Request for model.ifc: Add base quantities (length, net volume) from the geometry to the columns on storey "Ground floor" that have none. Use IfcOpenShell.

First a look at what the model holds.

```python
import ifcopenshell
import ifcopenshell.util.element
import ifcopenshell.util.unit

model = ifcopenshell.open("model.ifc")
print(model.schema)
for unit_type in ("LENGTHUNIT", "AREAUNIT", "VOLUMEUNIT"):
    print(unit_type, ifcopenshell.util.unit.calculate_unit_scale(model, unit_type))
storey = next(s for s in model.by_type("IfcBuildingStorey") if s.Name == "Ground floor")
columns = [e for e in ifcopenshell.util.element.get_decomposition(storey) if e.is_a("IfcColumn")]
for e in sorted(columns, key=lambda e: e.id()):
    print(e.id(), e.is_a(), e.Name, list(ifcopenshell.util.element.get_psets(e, qtos_only=True)), sep=" | ")
```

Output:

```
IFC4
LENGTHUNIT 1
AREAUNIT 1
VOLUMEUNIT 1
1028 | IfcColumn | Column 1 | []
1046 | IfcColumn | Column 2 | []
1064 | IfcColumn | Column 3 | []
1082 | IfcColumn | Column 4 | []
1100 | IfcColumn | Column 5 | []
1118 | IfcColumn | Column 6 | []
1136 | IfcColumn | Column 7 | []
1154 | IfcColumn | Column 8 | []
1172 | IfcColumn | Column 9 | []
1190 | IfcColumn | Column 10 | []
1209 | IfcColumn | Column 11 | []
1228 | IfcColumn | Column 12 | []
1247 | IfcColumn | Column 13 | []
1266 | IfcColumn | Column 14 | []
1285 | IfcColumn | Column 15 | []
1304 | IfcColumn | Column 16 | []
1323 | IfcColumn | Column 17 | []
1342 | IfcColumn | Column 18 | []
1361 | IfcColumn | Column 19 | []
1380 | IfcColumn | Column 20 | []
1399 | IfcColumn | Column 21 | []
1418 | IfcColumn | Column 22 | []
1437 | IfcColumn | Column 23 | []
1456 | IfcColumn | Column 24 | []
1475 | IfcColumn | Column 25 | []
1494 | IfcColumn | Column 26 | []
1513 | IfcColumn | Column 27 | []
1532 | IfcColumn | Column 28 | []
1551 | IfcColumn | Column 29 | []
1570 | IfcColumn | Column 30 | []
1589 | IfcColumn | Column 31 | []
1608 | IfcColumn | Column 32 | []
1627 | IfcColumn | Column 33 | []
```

```python
import ifcopenshell
import ifcopenshell.api.pset
import ifcopenshell.geom
import ifcopenshell.util.element
import ifcopenshell.util.shape
import ifcopenshell.util.unit

model = ifcopenshell.open("model.ifc")
unit_scale = ifcopenshell.util.unit.calculate_unit_scale(model)
volume_scale = ifcopenshell.util.unit.calculate_unit_scale(model, "VOLUMEUNIT")
settings = ifcopenshell.geom.settings()

storey = next(s for s in model.by_type("IfcBuildingStorey") if s.Name == "Ground floor")
columns = [e for e in ifcopenshell.util.element.get_decomposition(storey) if e.is_a("IfcColumn")]

for e in sorted(columns, key=lambda e: e.id()):
    if ifcopenshell.util.element.get_psets(e, qtos_only=True, should_inherit=False):
        continue
    # Geometry comes back in metres, in the element's own axes.
    shape = ifcopenshell.geom.create_shape(settings, e)
    values = {
        "Length": ifcopenshell.util.shape.get_z(shape.geometry) / unit_scale,
        "NetVolume": ifcopenshell.util.shape.get_volume(shape.geometry) / volume_scale,
    }
    qto = ifcopenshell.api.pset.add_qto(model, product=e, name="Qto_ColumnBaseQuantities")
    ifcopenshell.api.pset.edit_qto(model, qto=qto, properties=values)
    print(e.id(), {k: round(v, 3) for k, v in values.items()})

model.write("model_updated.ifc")
```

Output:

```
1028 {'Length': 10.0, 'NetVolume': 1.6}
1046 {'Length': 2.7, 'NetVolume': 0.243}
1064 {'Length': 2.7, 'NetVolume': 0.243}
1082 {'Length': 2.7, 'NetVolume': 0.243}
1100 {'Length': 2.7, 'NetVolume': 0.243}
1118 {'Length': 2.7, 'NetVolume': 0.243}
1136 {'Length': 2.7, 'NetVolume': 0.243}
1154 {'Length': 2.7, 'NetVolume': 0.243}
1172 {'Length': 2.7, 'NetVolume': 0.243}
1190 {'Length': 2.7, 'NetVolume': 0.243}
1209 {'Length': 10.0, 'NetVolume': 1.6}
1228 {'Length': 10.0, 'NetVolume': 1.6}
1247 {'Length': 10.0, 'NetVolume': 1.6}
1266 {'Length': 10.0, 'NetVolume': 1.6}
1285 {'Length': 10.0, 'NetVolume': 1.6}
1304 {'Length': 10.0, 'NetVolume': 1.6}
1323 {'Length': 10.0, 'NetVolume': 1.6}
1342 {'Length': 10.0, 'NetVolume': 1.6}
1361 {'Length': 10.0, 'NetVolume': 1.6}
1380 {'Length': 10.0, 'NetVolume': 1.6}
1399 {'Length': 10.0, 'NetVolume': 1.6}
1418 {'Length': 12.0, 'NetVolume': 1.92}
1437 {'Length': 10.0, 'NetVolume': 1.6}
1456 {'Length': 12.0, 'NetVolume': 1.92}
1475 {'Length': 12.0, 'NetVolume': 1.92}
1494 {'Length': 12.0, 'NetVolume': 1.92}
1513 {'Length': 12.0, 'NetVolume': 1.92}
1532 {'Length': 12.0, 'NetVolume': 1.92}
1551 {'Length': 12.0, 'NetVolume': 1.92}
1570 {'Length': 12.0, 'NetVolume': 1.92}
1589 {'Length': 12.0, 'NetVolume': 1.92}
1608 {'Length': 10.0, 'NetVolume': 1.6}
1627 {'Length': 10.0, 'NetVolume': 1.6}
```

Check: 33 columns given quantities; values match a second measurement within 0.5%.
